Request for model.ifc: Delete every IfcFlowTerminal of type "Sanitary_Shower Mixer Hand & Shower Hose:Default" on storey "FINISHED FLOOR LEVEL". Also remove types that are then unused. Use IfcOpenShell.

First a look at what the model holds.

```python
import ifcopenshell
import ifcopenshell.util.element

model = ifcopenshell.open("model.ifc")
print(model.schema)
storey = next(s for s in model.by_type("IfcBuildingStorey") if s.Name == "FINISHED FLOOR LEVEL")
terminals = [e for e in ifcopenshell.util.element.get_decomposition(storey) if e.is_a("IfcFlowTerminal")]
seen = {}
for e in terminals:
    element_type = ifcopenshell.util.element.get_type(e)
    name = element_type.Name if element_type not in (None, e) else None
    seen[name] = seen.get(name, 0) + 1
for name, count in sorted(seen.items(), key=str):
    print(count, "x", name)
```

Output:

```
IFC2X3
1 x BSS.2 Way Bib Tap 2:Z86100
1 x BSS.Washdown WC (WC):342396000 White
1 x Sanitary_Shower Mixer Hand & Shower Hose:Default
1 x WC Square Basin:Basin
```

```python
import ifcopenshell
import ifcopenshell.api.root
import ifcopenshell.util.element

model = ifcopenshell.open("model.ifc")

storey = next(s for s in model.by_type("IfcBuildingStorey") if s.Name == "FINISHED FLOOR LEVEL")
terminals = [e for e in ifcopenshell.util.element.get_decomposition(storey) if e.is_a("IfcFlowTerminal")]
targets = [e for e in terminals if (t := ifcopenshell.util.element.get_type(e)) not in (None, e) and t.Name == "Sanitary_Shower Mixer Hand & Shower Hose:Default"]
types = {ifcopenshell.util.element.get_type(e) for e in targets} - {None, *targets}

for e in targets:
    ifcopenshell.api.root.remove_product(model, product=e)
print(len(targets), "removed")

unused = [t for t in types if not ifcopenshell.util.element.get_types(t)]
for t in unused:
    ifcopenshell.api.root.remove_product(model, product=t)
print(len(unused), "unused types removed")

model.write("model-out.ifc")
```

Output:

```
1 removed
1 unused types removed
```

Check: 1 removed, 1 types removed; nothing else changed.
